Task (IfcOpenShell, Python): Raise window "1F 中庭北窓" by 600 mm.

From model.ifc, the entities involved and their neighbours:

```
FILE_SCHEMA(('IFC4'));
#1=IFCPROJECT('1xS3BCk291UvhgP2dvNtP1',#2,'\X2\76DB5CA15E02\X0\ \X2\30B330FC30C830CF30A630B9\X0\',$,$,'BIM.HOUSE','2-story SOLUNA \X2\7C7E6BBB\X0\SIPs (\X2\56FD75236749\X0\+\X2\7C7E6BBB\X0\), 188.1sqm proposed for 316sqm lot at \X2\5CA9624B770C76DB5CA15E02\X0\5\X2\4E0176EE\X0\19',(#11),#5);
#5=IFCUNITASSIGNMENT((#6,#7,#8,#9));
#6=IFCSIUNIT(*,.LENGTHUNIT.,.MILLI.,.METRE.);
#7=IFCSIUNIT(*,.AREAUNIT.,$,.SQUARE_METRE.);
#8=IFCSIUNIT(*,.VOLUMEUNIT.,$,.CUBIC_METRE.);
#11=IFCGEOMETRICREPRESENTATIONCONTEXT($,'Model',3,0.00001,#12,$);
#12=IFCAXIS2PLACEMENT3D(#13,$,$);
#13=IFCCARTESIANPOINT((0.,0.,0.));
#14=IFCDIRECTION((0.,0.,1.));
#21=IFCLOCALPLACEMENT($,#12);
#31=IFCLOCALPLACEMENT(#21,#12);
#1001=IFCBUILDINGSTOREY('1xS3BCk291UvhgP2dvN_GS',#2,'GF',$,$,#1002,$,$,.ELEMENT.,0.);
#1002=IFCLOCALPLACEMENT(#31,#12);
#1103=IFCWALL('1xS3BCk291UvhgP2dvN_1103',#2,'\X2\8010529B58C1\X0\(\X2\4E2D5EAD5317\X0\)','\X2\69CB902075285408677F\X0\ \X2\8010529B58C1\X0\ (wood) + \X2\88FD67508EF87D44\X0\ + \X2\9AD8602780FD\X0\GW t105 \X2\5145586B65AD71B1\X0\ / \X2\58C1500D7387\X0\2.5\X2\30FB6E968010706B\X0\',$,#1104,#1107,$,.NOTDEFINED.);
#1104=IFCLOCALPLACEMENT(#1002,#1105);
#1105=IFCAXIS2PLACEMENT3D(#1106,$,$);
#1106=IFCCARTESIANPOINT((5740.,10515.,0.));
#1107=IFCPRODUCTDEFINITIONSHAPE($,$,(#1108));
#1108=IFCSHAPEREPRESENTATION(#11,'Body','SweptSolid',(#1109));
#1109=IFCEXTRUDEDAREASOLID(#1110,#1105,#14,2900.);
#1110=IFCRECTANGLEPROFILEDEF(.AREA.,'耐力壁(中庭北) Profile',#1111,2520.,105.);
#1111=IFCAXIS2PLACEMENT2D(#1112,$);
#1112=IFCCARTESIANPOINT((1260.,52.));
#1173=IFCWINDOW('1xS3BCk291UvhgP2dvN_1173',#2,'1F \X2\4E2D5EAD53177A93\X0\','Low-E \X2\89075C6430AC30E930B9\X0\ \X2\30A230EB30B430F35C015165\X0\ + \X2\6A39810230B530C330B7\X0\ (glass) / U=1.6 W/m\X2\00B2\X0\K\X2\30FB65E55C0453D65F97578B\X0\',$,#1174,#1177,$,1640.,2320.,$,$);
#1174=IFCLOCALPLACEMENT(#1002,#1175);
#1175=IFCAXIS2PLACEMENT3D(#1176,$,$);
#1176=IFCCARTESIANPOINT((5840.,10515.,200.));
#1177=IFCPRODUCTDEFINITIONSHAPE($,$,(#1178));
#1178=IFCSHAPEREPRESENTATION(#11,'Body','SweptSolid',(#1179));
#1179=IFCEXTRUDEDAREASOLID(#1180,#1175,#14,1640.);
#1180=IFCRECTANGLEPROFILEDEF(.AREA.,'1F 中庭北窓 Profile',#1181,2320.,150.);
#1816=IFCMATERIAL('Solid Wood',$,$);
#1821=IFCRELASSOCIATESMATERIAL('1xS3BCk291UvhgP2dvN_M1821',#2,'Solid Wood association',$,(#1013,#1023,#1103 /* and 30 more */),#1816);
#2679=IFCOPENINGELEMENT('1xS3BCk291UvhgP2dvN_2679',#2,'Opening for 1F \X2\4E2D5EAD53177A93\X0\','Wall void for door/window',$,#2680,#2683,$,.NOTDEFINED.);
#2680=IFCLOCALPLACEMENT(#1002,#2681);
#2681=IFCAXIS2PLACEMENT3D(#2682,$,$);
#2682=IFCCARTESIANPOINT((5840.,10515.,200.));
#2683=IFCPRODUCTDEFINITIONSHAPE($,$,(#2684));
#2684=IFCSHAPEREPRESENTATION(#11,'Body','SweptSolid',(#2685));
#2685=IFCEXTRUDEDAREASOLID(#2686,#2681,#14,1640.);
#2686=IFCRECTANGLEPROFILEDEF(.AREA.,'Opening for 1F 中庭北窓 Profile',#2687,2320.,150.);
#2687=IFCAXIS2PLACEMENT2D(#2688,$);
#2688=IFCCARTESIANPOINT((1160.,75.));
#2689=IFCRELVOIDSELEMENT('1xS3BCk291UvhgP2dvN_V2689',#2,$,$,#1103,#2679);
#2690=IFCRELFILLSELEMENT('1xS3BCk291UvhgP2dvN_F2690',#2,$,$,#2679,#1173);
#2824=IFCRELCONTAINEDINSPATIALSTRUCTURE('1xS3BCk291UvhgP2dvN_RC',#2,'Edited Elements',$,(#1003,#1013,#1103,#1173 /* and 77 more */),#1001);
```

```python
import numpy as np
import ifcopenshell
import ifcopenshell.api.geometry
import ifcopenshell.util.placement
import ifcopenshell.util.unit

model = ifcopenshell.open("model.ifc")
unit_scale = ifcopenshell.util.unit.calculate_unit_scale(model)

window = model.by_guid("1xS3BCk291UvhgP2dvN_1173")
opening = window.FillsVoids[0].RelatingOpeningElement
dz = 600.0

shift = np.array([0.0, 0.0, dz])
# The window is not placed relative to its opening, so move both.
for product in (opening, window):
    matrix = ifcopenshell.util.placement.get_local_placement(product.ObjectPlacement)
    matrix[:3, 3] += shift
    ifcopenshell.api.geometry.edit_object_placement(model, product=product, matrix=matrix, is_si=False)

print(f"moved by {dz * unit_scale:+.3f} m")

model.write("model_edited.ifc")
```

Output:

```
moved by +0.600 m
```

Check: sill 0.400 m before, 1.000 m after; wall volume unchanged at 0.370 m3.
